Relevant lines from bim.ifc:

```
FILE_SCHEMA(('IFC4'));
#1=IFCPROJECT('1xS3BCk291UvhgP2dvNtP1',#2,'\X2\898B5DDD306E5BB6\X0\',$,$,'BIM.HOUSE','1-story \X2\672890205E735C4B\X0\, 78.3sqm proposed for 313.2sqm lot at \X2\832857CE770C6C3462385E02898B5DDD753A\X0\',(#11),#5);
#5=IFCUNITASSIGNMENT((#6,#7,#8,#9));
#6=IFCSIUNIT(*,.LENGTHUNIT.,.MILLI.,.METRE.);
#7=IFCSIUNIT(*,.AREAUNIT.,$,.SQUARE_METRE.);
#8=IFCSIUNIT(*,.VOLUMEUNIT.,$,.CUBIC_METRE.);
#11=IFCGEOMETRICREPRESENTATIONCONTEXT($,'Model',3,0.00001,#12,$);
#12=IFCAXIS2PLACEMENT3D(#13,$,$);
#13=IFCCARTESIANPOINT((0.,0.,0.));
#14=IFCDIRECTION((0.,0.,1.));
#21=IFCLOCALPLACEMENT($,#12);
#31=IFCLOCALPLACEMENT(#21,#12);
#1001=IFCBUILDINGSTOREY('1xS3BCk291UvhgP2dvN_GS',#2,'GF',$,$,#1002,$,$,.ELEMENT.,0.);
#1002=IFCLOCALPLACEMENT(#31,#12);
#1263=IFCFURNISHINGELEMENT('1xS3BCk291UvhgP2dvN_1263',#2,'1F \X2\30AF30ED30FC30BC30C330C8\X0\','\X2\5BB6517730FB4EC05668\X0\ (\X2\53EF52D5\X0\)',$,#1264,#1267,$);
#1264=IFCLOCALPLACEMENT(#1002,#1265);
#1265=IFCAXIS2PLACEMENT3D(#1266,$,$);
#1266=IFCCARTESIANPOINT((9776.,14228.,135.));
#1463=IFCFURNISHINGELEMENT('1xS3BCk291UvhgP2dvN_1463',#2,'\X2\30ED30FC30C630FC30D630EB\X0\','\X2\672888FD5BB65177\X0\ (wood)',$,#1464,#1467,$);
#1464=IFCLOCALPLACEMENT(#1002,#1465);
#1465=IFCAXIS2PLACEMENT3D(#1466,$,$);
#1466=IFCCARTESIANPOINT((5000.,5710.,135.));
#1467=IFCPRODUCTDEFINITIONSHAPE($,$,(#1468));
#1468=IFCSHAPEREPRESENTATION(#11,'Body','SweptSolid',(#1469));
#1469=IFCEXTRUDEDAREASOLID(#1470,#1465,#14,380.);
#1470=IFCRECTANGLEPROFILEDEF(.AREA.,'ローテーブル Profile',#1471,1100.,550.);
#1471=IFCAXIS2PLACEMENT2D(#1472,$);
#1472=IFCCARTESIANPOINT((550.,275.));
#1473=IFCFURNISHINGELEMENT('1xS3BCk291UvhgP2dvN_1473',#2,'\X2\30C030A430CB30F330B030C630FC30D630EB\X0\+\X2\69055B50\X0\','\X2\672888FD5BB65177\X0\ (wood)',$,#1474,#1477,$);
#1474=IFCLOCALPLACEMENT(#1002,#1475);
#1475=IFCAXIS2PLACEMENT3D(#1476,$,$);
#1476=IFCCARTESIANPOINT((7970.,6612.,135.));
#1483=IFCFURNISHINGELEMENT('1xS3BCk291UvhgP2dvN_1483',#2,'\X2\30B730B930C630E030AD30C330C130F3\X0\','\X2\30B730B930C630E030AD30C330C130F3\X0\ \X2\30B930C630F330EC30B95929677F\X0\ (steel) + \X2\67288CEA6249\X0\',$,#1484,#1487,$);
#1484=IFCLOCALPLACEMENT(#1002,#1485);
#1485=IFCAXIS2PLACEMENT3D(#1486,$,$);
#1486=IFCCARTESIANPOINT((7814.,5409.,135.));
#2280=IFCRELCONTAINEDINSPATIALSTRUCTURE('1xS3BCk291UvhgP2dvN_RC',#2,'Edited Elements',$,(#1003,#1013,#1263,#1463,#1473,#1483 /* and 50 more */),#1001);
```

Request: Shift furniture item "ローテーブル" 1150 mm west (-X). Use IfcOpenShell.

```python
import ifcopenshell
import ifcopenshell.api.geometry
import ifcopenshell.util.placement
import ifcopenshell.util.unit

model = ifcopenshell.open("bim.ifc")
unit_scale = ifcopenshell.util.unit.calculate_unit_scale(model)

item = model.by_id(1463)
matrix = ifcopenshell.util.placement.get_local_placement(item.ObjectPlacement)
matrix[0, 3] -= 1.15 / unit_scale
ifcopenshell.api.geometry.edit_object_placement(model, product=item, matrix=matrix, is_si=False)

print(ifcopenshell.util.placement.get_local_placement(item.ObjectPlacement).round(3) + 0.0)

model.write("bim_rev.ifc")
```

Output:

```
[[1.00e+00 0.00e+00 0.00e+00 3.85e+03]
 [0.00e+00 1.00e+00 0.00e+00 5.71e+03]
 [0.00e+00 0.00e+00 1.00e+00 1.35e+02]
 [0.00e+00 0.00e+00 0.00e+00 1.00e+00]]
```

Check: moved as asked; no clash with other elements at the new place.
